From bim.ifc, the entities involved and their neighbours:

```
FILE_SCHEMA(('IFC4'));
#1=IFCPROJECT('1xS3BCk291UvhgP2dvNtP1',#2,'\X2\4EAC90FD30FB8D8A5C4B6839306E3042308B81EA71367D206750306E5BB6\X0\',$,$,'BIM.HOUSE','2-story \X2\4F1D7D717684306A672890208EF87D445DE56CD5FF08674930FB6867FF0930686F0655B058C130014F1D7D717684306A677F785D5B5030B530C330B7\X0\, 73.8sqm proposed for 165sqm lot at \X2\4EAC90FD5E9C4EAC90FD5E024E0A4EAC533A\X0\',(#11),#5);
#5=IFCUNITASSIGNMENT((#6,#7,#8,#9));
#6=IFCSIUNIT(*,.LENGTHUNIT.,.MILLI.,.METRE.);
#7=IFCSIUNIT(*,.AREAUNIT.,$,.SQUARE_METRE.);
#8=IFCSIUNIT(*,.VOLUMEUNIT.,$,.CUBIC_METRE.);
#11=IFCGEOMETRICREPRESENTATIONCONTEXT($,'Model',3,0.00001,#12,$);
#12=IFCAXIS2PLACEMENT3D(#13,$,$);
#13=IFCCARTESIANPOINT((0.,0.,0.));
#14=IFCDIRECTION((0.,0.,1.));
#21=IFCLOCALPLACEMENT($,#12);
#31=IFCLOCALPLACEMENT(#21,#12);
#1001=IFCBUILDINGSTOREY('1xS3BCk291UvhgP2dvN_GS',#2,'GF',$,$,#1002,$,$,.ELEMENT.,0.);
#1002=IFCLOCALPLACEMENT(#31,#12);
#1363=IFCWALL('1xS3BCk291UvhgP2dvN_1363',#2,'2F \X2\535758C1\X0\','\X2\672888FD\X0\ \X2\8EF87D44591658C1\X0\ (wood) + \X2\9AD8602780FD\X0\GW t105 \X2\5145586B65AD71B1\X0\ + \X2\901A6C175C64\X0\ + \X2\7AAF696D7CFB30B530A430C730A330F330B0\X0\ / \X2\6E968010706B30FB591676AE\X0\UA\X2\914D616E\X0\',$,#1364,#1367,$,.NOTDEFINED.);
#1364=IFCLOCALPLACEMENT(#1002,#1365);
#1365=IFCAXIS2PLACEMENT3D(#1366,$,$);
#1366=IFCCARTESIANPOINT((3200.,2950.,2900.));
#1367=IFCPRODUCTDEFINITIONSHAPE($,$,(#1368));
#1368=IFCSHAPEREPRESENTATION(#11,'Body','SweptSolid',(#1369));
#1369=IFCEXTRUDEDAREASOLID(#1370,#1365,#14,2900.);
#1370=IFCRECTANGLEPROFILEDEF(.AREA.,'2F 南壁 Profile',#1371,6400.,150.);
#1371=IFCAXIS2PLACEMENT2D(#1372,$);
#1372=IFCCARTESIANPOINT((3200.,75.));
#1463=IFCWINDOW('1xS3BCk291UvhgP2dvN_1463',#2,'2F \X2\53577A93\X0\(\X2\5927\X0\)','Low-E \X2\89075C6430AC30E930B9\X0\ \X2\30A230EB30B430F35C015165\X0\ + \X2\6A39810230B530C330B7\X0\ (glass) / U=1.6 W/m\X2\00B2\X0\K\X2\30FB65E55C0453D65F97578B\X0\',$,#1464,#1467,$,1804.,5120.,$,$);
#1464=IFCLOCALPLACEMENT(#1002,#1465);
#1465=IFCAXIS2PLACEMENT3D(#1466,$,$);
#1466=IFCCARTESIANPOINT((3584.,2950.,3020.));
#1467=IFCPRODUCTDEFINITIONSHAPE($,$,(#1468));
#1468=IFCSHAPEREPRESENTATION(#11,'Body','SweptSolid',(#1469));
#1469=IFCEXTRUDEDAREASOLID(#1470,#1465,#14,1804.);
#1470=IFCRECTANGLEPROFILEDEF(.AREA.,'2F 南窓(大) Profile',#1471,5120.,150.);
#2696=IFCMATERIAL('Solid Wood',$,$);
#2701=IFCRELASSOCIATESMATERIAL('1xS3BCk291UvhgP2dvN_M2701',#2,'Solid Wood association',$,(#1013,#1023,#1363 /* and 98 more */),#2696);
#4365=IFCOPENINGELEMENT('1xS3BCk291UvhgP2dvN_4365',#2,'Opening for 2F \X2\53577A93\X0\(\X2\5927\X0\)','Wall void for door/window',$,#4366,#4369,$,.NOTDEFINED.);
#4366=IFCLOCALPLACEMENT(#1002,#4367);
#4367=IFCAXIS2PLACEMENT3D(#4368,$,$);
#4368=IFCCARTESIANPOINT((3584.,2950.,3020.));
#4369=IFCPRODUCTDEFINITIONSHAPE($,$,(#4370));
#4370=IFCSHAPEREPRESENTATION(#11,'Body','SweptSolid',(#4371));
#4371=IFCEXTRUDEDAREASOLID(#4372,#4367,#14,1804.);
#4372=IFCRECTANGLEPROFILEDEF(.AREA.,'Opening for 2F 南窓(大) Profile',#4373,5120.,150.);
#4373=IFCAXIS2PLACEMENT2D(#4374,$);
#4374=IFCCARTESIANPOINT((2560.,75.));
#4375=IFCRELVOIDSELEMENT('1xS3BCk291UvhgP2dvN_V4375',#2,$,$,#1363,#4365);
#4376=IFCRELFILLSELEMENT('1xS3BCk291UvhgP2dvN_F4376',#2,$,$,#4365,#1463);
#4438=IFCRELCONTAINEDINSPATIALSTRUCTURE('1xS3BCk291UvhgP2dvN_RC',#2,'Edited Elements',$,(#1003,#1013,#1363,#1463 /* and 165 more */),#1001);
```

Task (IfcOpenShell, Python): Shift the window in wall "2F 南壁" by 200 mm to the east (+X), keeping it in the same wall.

```python
import ifcopenshell
import ifcopenshell.api.geometry
import ifcopenshell.util.placement
import ifcopenshell.util.unit

model = ifcopenshell.open("bim.ifc")
unit_scale = ifcopenshell.util.unit.calculate_unit_scale(model)

window = model.by_guid("1xS3BCk291UvhgP2dvN_1463")
opening = window.FillsVoids[0].RelatingOpeningElement
wall = opening.VoidsElements[0].RelatingBuildingElement

wall_matrix = ifcopenshell.util.placement.get_local_placement(wall.ObjectPlacement)
shift = wall_matrix[:3, 0] * 0.2 / unit_scale
before = ifcopenshell.util.placement.get_local_placement(window.ObjectPlacement)[:3, 3].copy()

# The window is not placed relative to its opening, so move both.
for product in (opening, window):
    matrix = ifcopenshell.util.placement.get_local_placement(product.ObjectPlacement)
    matrix[:3, 3] += shift
    ifcopenshell.api.geometry.edit_object_placement(model, product=product, matrix=matrix, is_si=False)

after = ifcopenshell.util.placement.get_local_placement(window.ObjectPlacement)[:3, 3]
print("window moved by", (after - before).round(3) + 0.0)

model.write("bim_v2.ifc")
```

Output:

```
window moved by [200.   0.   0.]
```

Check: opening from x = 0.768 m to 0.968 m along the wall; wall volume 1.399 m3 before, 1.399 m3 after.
